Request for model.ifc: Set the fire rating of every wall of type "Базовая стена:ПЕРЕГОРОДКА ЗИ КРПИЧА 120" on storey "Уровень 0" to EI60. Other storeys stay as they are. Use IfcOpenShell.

First a look at what the model holds.

```python
import ifcopenshell
import ifcopenshell.util.element

model = ifcopenshell.open("model.ifc")
print(model.schema)
storey = next(s for s in model.by_type("IfcBuildingStorey") if s.Name == "Уровень 0")
walls = [e for e in ifcopenshell.util.element.get_decomposition(storey) if e.is_a("IfcWall")]
seen = {}
for e in walls:
    element_type = ifcopenshell.util.element.get_type(e)
    key = (element_type.Name if element_type != e and element_type else None, ifcopenshell.util.element.get_pset(e, "Pset_WallCommon", "FireRating"))
    seen[key] = seen.get(key, 0) + 1
for (name, value), count in sorted(seen.items(), key=str):
    print(count, "x", name, "|", value)
```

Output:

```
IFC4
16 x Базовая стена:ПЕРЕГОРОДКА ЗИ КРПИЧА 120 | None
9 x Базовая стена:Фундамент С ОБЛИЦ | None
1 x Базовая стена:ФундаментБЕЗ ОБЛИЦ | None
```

```python
import ifcopenshell
import ifcopenshell.api.pset
import ifcopenshell.util.element

model = ifcopenshell.open("model.ifc")

storey = next(s for s in model.by_type("IfcBuildingStorey") if s.Name == "Уровень 0")
walls = [e for e in ifcopenshell.util.element.get_decomposition(storey) if e.is_a("IfcWall")]

count = 0
for e in walls:
    element_type = ifcopenshell.util.element.get_type(e)
    if element_type in (None, e) or element_type.Name != "Базовая стена:ПЕРЕГОРОДКА ЗИ КРПИЧА 120":
        continue
    # add_pset returns the element's existing set when there is one.
    pset = ifcopenshell.api.pset.add_pset(model, product=e, name="Pset_WallCommon")
    ifcopenshell.api.pset.edit_pset(model, pset=pset, properties={"FireRating": "EI60"})
    count += 1

print(count, "walls updated")

model.write("model_edited.ifc")
```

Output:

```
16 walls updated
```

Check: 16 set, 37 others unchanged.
